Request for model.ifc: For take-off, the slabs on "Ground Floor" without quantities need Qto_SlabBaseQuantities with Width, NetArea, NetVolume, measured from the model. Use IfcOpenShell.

First a look at what the model holds.

```python
import ifcopenshell
import ifcopenshell.util.element
import ifcopenshell.util.unit

model = ifcopenshell.open("model.ifc")
print(model.schema)
for unit_type in ("LENGTHUNIT", "AREAUNIT", "VOLUMEUNIT"):
    print(unit_type, ifcopenshell.util.unit.calculate_unit_scale(model, unit_type))
storey = next(s for s in model.by_type("IfcBuildingStorey") if s.Name == "Ground Floor")
slabs = [e for e in ifcopenshell.util.element.get_decomposition(storey) if e.is_a("IfcSlab")]
for e in sorted(slabs, key=lambda e: e.id()):
    print(e.id(), e.is_a(), e.Name, list(ifcopenshell.util.element.get_psets(e, qtos_only=True)), sep=" | ")
```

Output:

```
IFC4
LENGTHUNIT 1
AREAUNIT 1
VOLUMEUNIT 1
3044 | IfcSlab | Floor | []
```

```python
import ifcopenshell
import ifcopenshell.api.pset
import ifcopenshell.geom
import ifcopenshell.util.element
import ifcopenshell.util.shape
import ifcopenshell.util.unit

model = ifcopenshell.open("model.ifc")
unit_scale = ifcopenshell.util.unit.calculate_unit_scale(model)
area_scale = ifcopenshell.util.unit.calculate_unit_scale(model, "AREAUNIT")
volume_scale = ifcopenshell.util.unit.calculate_unit_scale(model, "VOLUMEUNIT")
settings = ifcopenshell.geom.settings()

storey = next(s for s in model.by_type("IfcBuildingStorey") if s.Name == "Ground Floor")
slabs = [e for e in ifcopenshell.util.element.get_decomposition(storey) if e.is_a("IfcSlab")]

for e in sorted(slabs, key=lambda e: e.id()):
    if ifcopenshell.util.element.get_psets(e, qtos_only=True, should_inherit=False):
        continue
    # Geometry comes back in metres, in the element's own axes.
    shape = ifcopenshell.geom.create_shape(settings, e)
    values = {
        "Width": ifcopenshell.util.shape.get_z(shape.geometry) / unit_scale,
        "NetArea": ifcopenshell.util.shape.get_footprint_area(shape.geometry) / area_scale,
        "NetVolume": ifcopenshell.util.shape.get_volume(shape.geometry) / volume_scale,
    }
    qto = ifcopenshell.api.pset.add_qto(model, product=e, name="Qto_SlabBaseQuantities")
    ifcopenshell.api.pset.edit_qto(model, qto=qto, properties=values)
    print(e.id(), {k: round(v, 3) for k, v in values.items()})

model.write("model_rev.ifc")
```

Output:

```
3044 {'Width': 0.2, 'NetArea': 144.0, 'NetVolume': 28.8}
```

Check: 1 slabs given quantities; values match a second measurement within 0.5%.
